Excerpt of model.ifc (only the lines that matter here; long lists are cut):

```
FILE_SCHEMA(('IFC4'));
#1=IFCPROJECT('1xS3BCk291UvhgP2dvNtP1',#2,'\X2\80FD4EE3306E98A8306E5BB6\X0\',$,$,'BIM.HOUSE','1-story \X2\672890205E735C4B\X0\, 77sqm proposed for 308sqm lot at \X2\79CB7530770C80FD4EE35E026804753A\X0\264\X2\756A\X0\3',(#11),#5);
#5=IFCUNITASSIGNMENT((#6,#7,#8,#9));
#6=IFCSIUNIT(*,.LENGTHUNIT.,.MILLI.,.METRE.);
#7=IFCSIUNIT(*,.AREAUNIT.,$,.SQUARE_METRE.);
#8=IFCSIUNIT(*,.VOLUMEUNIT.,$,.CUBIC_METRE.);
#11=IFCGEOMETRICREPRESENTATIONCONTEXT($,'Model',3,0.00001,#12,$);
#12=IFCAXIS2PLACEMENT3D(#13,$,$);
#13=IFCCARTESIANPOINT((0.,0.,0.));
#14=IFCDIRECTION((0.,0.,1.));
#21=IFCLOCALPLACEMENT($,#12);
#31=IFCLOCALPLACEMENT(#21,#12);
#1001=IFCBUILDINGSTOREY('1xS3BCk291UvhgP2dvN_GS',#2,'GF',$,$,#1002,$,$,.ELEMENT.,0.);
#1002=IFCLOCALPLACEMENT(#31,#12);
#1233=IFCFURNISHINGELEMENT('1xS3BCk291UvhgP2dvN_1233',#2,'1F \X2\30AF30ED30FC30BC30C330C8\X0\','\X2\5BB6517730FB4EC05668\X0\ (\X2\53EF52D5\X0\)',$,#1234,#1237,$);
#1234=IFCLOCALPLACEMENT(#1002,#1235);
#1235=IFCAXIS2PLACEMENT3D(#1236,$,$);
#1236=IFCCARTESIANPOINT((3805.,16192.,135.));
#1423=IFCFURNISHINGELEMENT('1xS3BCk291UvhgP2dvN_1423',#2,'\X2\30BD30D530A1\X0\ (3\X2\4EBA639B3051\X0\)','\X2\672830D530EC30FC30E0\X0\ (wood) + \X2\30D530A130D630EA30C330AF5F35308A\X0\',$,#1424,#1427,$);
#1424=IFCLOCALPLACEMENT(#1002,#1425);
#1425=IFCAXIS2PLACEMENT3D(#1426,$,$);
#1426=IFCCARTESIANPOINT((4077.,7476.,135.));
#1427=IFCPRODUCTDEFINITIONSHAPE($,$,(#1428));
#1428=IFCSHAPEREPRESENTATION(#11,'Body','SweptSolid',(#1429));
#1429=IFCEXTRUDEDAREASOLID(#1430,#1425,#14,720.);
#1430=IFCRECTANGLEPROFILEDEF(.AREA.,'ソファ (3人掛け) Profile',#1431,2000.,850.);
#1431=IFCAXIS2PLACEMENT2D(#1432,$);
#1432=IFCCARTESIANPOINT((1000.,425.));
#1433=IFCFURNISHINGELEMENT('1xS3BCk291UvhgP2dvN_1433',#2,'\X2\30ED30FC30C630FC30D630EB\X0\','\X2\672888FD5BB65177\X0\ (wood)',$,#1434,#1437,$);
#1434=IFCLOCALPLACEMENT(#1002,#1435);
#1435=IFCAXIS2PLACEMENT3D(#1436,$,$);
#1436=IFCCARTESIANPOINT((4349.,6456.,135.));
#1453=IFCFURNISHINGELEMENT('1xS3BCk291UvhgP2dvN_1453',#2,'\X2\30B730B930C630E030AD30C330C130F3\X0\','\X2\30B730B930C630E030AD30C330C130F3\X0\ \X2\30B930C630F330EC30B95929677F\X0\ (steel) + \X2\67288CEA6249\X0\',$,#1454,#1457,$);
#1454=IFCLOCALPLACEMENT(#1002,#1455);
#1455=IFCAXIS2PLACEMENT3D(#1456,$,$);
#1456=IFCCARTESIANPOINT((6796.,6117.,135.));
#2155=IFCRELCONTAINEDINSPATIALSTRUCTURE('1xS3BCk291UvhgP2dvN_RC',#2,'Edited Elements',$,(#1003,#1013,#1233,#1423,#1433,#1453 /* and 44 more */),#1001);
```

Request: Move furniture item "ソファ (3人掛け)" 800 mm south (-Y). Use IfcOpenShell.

```python
import ifcopenshell
import ifcopenshell.api.geometry
import ifcopenshell.util.placement
import ifcopenshell.util.unit

model = ifcopenshell.open("model.ifc")
unit_scale = ifcopenshell.util.unit.calculate_unit_scale(model)

item = model.by_guid("1xS3BCk291UvhgP2dvN_1423")
matrix = ifcopenshell.util.placement.get_local_placement(item.ObjectPlacement)
matrix[1, 3] -= 0.8 / unit_scale
ifcopenshell.api.geometry.edit_object_placement(model, product=item, matrix=matrix, is_si=False)

print(ifcopenshell.util.placement.get_local_placement(item.ObjectPlacement).round(3) + 0.0)

model.write("model_v2.ifc")
```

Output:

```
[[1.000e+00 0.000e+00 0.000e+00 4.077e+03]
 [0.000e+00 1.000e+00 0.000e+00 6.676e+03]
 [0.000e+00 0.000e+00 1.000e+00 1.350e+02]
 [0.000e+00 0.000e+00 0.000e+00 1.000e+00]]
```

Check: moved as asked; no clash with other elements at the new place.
